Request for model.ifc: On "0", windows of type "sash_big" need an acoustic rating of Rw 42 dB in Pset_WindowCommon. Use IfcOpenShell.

First a look at what the model holds.

```python
import ifcopenshell
import ifcopenshell.util.element

model = ifcopenshell.open("model.ifc")
print(model.schema)
storey = next(s for s in model.by_type("IfcBuildingStorey") if s.Name == "0")
windows = [e for e in ifcopenshell.util.element.get_decomposition(storey) if e.is_a("IfcWindow")]
seen = {}
for e in windows:
    element_type = ifcopenshell.util.element.get_type(e)
    key = (element_type.Name if element_type != e and element_type else None, ifcopenshell.util.element.get_pset(e, "Pset_WindowCommon", "AcousticRating"))
    seen[key] = seen.get(key, 0) + 1
for (name, value), count in sorted(seen.items(), key=str):
    print(count, "x", name, "|", value)
```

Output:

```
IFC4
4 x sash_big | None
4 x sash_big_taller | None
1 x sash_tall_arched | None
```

```python
import ifcopenshell
import ifcopenshell.api.pset
import ifcopenshell.util.element

model = ifcopenshell.open("model.ifc")

storey = next(s for s in model.by_type("IfcBuildingStorey") if s.Name == "0")
windows = [e for e in ifcopenshell.util.element.get_decomposition(storey) if e.is_a("IfcWindow")]

count = 0
for e in windows:
    element_type = ifcopenshell.util.element.get_type(e)
    if element_type in (None, e) or element_type.Name != "sash_big":
        continue
    # add_pset returns the element's existing set when there is one.
    pset = ifcopenshell.api.pset.add_pset(model, product=e, name="Pset_WindowCommon")
    ifcopenshell.api.pset.edit_pset(model, pset=pset, properties={"AcousticRating": "Rw 42 dB"})
    count += 1

print(count, "windows updated")

model.write("model_v2.ifc")
```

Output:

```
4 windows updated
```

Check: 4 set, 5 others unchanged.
